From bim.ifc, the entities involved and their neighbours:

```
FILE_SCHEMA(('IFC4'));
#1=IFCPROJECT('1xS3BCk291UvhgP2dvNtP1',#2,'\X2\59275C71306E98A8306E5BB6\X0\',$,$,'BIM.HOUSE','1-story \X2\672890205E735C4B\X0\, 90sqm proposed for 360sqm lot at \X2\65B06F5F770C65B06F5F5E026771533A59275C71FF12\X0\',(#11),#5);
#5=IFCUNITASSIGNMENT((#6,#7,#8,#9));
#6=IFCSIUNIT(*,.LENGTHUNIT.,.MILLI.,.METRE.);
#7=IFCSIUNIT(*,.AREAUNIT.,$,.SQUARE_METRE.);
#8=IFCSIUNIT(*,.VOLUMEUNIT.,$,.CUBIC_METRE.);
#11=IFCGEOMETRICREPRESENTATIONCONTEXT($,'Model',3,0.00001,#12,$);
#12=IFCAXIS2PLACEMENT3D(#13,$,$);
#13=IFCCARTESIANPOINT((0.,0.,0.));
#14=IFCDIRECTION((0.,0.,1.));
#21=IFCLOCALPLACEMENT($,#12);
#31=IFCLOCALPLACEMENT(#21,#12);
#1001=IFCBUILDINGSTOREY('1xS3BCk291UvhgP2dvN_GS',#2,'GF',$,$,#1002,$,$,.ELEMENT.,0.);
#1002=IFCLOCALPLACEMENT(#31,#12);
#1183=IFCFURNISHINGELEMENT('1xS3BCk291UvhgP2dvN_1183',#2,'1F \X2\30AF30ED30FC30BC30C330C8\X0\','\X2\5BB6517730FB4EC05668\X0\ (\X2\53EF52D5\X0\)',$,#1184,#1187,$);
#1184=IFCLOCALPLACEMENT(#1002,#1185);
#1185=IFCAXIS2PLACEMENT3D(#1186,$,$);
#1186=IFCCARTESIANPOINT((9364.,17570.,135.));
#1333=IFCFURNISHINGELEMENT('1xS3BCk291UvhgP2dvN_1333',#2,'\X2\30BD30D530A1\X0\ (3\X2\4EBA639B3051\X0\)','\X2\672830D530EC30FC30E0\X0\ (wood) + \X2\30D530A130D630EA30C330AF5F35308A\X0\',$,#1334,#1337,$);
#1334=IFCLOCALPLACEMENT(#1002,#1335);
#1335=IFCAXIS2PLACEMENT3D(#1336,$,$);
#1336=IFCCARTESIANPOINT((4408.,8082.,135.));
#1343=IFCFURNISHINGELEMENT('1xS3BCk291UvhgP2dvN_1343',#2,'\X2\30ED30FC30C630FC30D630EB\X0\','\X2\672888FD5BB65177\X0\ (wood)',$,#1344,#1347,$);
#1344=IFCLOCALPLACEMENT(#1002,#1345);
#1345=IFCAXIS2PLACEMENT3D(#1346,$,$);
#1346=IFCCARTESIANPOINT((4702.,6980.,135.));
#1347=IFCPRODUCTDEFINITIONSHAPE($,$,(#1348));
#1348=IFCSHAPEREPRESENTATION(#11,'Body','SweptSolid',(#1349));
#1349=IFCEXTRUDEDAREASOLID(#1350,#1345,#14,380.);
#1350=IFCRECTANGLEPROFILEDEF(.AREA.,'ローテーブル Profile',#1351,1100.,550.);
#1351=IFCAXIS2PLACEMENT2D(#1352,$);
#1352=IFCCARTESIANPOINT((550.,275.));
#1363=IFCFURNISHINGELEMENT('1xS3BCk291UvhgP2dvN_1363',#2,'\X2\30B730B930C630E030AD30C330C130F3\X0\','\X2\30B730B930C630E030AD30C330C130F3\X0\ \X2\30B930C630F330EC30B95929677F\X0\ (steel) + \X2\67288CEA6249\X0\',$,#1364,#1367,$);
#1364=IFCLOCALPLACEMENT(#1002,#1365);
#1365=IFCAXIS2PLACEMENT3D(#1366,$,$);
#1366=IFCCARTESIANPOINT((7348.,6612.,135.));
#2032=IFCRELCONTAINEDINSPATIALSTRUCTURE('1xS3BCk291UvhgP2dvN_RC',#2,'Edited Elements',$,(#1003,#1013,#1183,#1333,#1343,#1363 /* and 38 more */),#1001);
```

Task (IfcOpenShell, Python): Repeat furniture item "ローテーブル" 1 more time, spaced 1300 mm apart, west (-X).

```python
import numpy as np
import ifcopenshell
import ifcopenshell.api.geometry
import ifcopenshell.api.root
import ifcopenshell.util.element
import ifcopenshell.util.placement

model = ifcopenshell.open("bim.ifc")


def reuse_history(source, copy):
    """copy_class also copies each property set's owner history, people and application; keep the originals."""
    for rel in copy.IsDefinedBy:
        if rel.is_a("IfcRelDefinesByProperties") and (history := rel.RelatingPropertyDefinition.OwnerHistory):
            rel.RelatingPropertyDefinition.OwnerHistory = source.OwnerHistory
            ifcopenshell.util.element.remove_deep2(model, history)


source = model.by_guid("1xS3BCk291UvhgP2dvN_1343")
base = ifcopenshell.util.placement.get_local_placement(source.ObjectPlacement)
step = np.array([-1.0, 0.0, 0.0]) * 1300.0

for i in range(1, 2):
    copy = ifcopenshell.api.root.copy_class(model, product=source)
    copy.Representation = ifcopenshell.util.element.copy_deep(
        model, source.Representation, exclude=["IfcGeometricRepresentationContext", "IfcRepresentationMap"]
    )
    reuse_history(source, copy)
    matrix = base.copy()
    matrix[:3, 3] += i * step
    print("added at", matrix[:3, 3].round(3) + 0.0)
    ifcopenshell.api.geometry.edit_object_placement(model, product=copy, matrix=matrix, is_si=False)

model.write("bim_edited.ifc")
```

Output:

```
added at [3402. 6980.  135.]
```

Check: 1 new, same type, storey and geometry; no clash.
